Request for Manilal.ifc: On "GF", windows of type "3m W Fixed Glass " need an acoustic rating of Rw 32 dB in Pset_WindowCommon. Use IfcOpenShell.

First a look at what the model holds.

```python
import ifcopenshell
import ifcopenshell.util.element

model = ifcopenshell.open("Manilal.ifc")
print(model.schema)
storey = next(s for s in model.by_type("IfcBuildingStorey") if s.Name == "GF")
windows = [e for e in ifcopenshell.util.element.get_decomposition(storey) if e.is_a("IfcWindow")]
seen = {}
for e in windows:
    element_type = ifcopenshell.util.element.get_type(e)
    key = (element_type.Name if element_type != e and element_type else None, ifcopenshell.util.element.get_pset(e, "Pset_WindowCommon", "AcousticRating"))
    seen[key] = seen.get(key, 0) + 1
for (name, value), count in sorted(seen.items(), key=str):
    print(count, "x", name, "|", value)
```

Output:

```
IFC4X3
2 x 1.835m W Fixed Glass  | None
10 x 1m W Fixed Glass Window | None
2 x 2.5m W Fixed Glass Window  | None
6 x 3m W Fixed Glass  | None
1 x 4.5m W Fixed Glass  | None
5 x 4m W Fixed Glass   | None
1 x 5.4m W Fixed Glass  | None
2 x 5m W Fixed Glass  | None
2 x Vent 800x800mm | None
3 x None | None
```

```python
import ifcopenshell
import ifcopenshell.api.pset
import ifcopenshell.util.element

model = ifcopenshell.open("Manilal.ifc")

storey = next(s for s in model.by_type("IfcBuildingStorey") if s.Name == "GF")
windows = [e for e in ifcopenshell.util.element.get_decomposition(storey) if e.is_a("IfcWindow")]

count = 0
for e in windows:
    element_type = ifcopenshell.util.element.get_type(e)
    if element_type in (None, e) or element_type.Name != "3m W Fixed Glass ":
        continue
    # add_pset returns the element's existing set when there is one.
    pset = ifcopenshell.api.pset.add_pset(model, product=e, name="Pset_WindowCommon")
    ifcopenshell.api.pset.edit_pset(model, pset=pset, properties={"AcousticRating": "Rw 32 dB"})
    count += 1

print(count, "windows updated")

model.write("Manilal_updated.ifc")
```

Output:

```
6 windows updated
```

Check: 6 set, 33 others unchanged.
